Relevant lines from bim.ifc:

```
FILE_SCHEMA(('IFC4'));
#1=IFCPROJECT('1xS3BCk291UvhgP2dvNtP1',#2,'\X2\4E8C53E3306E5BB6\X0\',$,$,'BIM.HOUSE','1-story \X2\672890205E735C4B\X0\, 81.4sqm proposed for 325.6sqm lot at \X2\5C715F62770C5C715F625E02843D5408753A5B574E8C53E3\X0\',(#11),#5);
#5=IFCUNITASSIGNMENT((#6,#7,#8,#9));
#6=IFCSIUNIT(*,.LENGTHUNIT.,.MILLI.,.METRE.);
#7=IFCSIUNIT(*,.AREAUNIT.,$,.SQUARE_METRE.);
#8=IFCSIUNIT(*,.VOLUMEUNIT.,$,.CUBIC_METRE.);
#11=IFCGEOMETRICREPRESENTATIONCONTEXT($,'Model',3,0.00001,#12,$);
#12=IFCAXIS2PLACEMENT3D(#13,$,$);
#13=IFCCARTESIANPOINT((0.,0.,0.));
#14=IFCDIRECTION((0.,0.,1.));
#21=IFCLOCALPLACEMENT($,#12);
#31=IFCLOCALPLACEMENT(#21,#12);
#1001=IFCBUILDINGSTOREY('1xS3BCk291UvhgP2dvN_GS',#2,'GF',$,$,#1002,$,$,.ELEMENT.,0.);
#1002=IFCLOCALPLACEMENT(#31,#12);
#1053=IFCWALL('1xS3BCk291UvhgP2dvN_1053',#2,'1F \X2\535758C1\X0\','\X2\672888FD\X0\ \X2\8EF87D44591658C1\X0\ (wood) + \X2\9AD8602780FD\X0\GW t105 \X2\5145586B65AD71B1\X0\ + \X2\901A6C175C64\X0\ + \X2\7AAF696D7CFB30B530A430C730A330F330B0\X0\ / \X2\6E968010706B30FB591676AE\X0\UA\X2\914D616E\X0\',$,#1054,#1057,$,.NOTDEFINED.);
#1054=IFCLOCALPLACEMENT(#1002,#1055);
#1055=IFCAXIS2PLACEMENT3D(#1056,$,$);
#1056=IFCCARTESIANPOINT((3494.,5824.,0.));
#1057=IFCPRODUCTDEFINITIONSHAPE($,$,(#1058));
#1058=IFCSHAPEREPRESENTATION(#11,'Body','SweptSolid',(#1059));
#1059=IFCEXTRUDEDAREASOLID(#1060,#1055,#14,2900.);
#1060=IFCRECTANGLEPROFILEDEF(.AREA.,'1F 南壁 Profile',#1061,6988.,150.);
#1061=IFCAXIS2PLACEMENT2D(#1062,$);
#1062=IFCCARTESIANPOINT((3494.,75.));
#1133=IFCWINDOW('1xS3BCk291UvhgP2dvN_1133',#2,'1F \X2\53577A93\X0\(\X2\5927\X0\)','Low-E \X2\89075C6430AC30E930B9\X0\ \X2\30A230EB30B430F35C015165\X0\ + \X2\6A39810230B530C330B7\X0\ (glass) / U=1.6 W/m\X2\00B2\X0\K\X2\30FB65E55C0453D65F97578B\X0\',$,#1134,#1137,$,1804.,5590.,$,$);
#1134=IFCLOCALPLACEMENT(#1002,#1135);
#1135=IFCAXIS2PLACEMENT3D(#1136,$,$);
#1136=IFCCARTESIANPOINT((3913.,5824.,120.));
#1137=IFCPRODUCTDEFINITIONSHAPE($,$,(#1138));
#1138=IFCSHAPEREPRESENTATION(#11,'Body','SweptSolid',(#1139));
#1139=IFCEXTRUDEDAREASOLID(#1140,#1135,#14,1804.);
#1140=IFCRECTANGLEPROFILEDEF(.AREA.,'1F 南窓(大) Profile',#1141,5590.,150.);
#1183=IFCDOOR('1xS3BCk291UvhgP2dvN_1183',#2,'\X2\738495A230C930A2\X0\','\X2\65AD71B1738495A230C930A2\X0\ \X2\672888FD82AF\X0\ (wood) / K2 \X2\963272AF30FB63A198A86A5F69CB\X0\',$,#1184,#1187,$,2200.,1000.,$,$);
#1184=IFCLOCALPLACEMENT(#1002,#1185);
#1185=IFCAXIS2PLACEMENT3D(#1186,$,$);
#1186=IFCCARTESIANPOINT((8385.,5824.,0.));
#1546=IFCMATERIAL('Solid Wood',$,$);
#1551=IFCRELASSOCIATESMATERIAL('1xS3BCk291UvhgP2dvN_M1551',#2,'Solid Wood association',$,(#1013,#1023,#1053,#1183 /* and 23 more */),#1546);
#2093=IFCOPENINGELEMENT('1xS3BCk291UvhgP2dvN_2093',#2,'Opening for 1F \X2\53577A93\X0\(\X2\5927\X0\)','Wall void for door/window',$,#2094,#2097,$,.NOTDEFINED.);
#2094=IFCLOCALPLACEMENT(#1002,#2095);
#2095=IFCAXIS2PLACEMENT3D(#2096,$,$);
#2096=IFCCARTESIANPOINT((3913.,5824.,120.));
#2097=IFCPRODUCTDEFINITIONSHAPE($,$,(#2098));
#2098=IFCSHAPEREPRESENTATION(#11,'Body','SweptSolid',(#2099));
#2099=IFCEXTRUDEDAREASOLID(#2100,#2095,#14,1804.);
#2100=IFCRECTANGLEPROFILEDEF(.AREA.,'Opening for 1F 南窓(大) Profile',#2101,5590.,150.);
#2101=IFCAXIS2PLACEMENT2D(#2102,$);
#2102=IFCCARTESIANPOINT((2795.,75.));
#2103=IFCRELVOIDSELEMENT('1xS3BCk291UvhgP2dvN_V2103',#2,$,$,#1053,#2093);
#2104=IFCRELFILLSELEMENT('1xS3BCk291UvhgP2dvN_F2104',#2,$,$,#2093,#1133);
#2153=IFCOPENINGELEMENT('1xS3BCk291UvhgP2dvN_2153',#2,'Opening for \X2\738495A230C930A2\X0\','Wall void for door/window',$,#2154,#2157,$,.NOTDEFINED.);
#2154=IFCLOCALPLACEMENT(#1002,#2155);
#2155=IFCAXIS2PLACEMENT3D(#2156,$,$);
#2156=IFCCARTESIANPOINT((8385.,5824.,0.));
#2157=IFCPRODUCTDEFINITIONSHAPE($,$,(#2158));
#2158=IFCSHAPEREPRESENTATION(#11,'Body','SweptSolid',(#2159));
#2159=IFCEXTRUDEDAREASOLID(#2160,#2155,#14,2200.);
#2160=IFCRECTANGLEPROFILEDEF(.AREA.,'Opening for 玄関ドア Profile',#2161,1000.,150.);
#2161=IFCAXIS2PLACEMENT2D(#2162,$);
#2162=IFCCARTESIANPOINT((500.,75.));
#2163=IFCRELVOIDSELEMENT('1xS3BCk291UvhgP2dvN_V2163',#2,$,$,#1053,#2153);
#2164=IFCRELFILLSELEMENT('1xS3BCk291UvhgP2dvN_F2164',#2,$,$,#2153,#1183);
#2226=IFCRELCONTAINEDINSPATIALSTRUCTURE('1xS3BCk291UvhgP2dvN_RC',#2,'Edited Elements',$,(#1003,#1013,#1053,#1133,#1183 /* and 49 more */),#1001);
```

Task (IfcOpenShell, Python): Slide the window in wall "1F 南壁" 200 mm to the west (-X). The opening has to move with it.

```python
import ifcopenshell
import ifcopenshell.api.geometry
import ifcopenshell.util.placement
import ifcopenshell.util.unit

model = ifcopenshell.open("bim.ifc")
unit_scale = ifcopenshell.util.unit.calculate_unit_scale(model)

window = model.by_id(1133)
opening = window.FillsVoids[0].RelatingOpeningElement
wall = opening.VoidsElements[0].RelatingBuildingElement

wall_matrix = ifcopenshell.util.placement.get_local_placement(wall.ObjectPlacement)
shift = wall_matrix[:3, 0] * -0.2 / unit_scale
before = ifcopenshell.util.placement.get_local_placement(window.ObjectPlacement)[:3, 3].copy()

# The window is not placed relative to its opening, so move both.
for product in (opening, window):
    matrix = ifcopenshell.util.placement.get_local_placement(product.ObjectPlacement)
    matrix[:3, 3] += shift
    ifcopenshell.api.geometry.edit_object_placement(model, product=product, matrix=matrix, is_si=False)

after = ifcopenshell.util.placement.get_local_placement(window.ObjectPlacement)[:3, 3]
print("window moved by", (after - before).round(3) + 0.0)

model.write("bim_edited.ifc")
```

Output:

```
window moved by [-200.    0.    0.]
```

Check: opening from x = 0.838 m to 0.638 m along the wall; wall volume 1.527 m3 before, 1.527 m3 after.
